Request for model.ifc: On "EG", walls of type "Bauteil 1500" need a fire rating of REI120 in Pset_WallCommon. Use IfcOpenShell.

First a look at what the model holds.

```python
import ifcopenshell
import ifcopenshell.util.element

model = ifcopenshell.open("model.ifc")
print(model.schema)
storey = next(s for s in model.by_type("IfcBuildingStorey") if s.Name == "EG")
walls = [e for e in ifcopenshell.util.element.get_decomposition(storey) if e.is_a("IfcWall")]
seen = {}
for e in walls:
    element_type = ifcopenshell.util.element.get_type(e)
    key = (element_type.Name if element_type != e and element_type else None, ifcopenshell.util.element.get_pset(e, "Pset_WallCommon", "FireRating"))
    seen[key] = seen.get(key, 0) + 1
for (name, value), count in sorted(seen.items(), key=str):
    print(count, "x", name, "|", value)
```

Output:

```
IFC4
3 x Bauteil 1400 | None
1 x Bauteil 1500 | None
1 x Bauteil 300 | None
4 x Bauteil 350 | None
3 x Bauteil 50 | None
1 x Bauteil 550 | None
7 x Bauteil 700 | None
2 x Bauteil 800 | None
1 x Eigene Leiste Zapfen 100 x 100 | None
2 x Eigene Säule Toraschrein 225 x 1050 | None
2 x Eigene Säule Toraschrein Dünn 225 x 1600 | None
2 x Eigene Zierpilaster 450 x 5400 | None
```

```python
import ifcopenshell
import ifcopenshell.api.pset
import ifcopenshell.util.element

model = ifcopenshell.open("model.ifc")

storey = next(s for s in model.by_type("IfcBuildingStorey") if s.Name == "EG")
walls = [e for e in ifcopenshell.util.element.get_decomposition(storey) if e.is_a("IfcWall")]

count = 0
for e in walls:
    element_type = ifcopenshell.util.element.get_type(e)
    if element_type in (None, e) or element_type.Name != "Bauteil 1500":
        continue
    # add_pset returns the element's existing set when there is one.
    pset = ifcopenshell.api.pset.add_pset(model, product=e, name="Pset_WallCommon")
    ifcopenshell.api.pset.edit_pset(model, pset=pset, properties={"FireRating": "REI120"})
    count += 1

print(count, "walls updated")

model.write("model-out.ifc")
```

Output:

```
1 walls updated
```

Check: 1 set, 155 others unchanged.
